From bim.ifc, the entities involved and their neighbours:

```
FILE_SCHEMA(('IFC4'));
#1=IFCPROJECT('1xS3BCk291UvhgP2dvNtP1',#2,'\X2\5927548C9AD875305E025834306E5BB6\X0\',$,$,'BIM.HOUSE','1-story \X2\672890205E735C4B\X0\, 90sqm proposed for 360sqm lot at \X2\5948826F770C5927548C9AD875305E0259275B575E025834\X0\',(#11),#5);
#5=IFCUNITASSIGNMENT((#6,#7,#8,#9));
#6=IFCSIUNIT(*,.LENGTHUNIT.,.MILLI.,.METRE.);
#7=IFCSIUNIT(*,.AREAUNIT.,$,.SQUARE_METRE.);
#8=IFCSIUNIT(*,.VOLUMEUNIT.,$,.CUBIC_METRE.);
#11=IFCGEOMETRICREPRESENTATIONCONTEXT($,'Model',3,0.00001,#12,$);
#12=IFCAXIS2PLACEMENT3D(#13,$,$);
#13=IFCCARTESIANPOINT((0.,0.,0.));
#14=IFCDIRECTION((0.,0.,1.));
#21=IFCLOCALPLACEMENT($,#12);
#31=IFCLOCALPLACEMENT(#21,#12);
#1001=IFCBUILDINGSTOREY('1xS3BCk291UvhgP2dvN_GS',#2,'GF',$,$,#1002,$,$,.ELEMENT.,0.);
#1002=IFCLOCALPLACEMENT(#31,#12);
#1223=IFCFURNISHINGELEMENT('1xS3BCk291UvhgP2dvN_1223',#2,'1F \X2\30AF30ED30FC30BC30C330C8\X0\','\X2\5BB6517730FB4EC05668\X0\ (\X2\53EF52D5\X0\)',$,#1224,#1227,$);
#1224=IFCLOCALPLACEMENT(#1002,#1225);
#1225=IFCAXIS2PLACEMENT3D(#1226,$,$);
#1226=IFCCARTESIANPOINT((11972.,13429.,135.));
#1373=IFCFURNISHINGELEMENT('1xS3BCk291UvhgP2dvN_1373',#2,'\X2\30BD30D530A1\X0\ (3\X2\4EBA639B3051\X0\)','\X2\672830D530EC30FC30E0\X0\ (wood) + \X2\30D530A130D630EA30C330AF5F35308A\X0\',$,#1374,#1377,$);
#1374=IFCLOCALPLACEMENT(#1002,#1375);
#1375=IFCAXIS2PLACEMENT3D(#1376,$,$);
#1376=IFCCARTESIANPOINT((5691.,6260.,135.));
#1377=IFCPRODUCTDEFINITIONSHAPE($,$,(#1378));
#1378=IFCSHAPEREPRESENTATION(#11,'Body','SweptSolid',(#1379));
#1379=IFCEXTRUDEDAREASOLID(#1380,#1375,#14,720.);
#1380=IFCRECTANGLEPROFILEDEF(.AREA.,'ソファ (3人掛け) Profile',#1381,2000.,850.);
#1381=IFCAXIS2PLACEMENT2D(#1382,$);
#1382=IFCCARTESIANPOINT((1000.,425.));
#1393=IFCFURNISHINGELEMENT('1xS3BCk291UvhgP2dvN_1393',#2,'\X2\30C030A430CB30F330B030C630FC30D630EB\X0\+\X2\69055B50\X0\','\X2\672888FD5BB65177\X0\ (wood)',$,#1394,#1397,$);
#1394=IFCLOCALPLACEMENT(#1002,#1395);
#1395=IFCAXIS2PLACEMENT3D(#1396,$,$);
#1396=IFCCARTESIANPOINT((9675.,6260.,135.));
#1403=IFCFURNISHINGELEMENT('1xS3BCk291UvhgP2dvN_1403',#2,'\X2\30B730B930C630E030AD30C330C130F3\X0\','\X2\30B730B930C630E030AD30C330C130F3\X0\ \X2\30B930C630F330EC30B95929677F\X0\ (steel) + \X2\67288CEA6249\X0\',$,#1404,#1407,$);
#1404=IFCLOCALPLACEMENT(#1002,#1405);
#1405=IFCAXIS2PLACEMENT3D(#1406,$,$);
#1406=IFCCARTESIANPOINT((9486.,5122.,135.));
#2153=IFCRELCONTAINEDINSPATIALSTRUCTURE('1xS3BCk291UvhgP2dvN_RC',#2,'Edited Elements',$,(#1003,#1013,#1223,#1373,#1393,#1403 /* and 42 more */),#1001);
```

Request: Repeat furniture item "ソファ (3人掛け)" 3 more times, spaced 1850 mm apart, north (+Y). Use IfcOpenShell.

```python
import numpy as np
import ifcopenshell
import ifcopenshell.api.geometry
import ifcopenshell.api.root
import ifcopenshell.util.element
import ifcopenshell.util.placement
import ifcopenshell.util.unit

model = ifcopenshell.open("bim.ifc")
unit_scale = ifcopenshell.util.unit.calculate_unit_scale(model)


def reuse_history(source, copy):
    """copy_class also copies each property set's owner history, people and application; keep the originals."""
    for rel in copy.IsDefinedBy:
        if rel.is_a("IfcRelDefinesByProperties") and (history := rel.RelatingPropertyDefinition.OwnerHistory):
            rel.RelatingPropertyDefinition.OwnerHistory = source.OwnerHistory
            ifcopenshell.util.element.remove_deep2(model, history)


source = model.by_id(1373)
base = ifcopenshell.util.placement.get_local_placement(source.ObjectPlacement)
step = np.array([0.0, 1.0, 0.0]) * 1.85 / unit_scale

for i in range(1, 4):
    copy = ifcopenshell.api.root.copy_class(model, product=source)
    copy.Representation = ifcopenshell.util.element.copy_deep(
        model, source.Representation, exclude=["IfcGeometricRepresentationContext", "IfcRepresentationMap"]
    )
    reuse_history(source, copy)
    matrix = base.copy()
    matrix[:3, 3] += i * step
    print("added at", matrix[:3, 3].round(3) + 0.0)
    ifcopenshell.api.geometry.edit_object_placement(model, product=copy, matrix=matrix, is_si=False)

model.write("bim_edited.ifc")
```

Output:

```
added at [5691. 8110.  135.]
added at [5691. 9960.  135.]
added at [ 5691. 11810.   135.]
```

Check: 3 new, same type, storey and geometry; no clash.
